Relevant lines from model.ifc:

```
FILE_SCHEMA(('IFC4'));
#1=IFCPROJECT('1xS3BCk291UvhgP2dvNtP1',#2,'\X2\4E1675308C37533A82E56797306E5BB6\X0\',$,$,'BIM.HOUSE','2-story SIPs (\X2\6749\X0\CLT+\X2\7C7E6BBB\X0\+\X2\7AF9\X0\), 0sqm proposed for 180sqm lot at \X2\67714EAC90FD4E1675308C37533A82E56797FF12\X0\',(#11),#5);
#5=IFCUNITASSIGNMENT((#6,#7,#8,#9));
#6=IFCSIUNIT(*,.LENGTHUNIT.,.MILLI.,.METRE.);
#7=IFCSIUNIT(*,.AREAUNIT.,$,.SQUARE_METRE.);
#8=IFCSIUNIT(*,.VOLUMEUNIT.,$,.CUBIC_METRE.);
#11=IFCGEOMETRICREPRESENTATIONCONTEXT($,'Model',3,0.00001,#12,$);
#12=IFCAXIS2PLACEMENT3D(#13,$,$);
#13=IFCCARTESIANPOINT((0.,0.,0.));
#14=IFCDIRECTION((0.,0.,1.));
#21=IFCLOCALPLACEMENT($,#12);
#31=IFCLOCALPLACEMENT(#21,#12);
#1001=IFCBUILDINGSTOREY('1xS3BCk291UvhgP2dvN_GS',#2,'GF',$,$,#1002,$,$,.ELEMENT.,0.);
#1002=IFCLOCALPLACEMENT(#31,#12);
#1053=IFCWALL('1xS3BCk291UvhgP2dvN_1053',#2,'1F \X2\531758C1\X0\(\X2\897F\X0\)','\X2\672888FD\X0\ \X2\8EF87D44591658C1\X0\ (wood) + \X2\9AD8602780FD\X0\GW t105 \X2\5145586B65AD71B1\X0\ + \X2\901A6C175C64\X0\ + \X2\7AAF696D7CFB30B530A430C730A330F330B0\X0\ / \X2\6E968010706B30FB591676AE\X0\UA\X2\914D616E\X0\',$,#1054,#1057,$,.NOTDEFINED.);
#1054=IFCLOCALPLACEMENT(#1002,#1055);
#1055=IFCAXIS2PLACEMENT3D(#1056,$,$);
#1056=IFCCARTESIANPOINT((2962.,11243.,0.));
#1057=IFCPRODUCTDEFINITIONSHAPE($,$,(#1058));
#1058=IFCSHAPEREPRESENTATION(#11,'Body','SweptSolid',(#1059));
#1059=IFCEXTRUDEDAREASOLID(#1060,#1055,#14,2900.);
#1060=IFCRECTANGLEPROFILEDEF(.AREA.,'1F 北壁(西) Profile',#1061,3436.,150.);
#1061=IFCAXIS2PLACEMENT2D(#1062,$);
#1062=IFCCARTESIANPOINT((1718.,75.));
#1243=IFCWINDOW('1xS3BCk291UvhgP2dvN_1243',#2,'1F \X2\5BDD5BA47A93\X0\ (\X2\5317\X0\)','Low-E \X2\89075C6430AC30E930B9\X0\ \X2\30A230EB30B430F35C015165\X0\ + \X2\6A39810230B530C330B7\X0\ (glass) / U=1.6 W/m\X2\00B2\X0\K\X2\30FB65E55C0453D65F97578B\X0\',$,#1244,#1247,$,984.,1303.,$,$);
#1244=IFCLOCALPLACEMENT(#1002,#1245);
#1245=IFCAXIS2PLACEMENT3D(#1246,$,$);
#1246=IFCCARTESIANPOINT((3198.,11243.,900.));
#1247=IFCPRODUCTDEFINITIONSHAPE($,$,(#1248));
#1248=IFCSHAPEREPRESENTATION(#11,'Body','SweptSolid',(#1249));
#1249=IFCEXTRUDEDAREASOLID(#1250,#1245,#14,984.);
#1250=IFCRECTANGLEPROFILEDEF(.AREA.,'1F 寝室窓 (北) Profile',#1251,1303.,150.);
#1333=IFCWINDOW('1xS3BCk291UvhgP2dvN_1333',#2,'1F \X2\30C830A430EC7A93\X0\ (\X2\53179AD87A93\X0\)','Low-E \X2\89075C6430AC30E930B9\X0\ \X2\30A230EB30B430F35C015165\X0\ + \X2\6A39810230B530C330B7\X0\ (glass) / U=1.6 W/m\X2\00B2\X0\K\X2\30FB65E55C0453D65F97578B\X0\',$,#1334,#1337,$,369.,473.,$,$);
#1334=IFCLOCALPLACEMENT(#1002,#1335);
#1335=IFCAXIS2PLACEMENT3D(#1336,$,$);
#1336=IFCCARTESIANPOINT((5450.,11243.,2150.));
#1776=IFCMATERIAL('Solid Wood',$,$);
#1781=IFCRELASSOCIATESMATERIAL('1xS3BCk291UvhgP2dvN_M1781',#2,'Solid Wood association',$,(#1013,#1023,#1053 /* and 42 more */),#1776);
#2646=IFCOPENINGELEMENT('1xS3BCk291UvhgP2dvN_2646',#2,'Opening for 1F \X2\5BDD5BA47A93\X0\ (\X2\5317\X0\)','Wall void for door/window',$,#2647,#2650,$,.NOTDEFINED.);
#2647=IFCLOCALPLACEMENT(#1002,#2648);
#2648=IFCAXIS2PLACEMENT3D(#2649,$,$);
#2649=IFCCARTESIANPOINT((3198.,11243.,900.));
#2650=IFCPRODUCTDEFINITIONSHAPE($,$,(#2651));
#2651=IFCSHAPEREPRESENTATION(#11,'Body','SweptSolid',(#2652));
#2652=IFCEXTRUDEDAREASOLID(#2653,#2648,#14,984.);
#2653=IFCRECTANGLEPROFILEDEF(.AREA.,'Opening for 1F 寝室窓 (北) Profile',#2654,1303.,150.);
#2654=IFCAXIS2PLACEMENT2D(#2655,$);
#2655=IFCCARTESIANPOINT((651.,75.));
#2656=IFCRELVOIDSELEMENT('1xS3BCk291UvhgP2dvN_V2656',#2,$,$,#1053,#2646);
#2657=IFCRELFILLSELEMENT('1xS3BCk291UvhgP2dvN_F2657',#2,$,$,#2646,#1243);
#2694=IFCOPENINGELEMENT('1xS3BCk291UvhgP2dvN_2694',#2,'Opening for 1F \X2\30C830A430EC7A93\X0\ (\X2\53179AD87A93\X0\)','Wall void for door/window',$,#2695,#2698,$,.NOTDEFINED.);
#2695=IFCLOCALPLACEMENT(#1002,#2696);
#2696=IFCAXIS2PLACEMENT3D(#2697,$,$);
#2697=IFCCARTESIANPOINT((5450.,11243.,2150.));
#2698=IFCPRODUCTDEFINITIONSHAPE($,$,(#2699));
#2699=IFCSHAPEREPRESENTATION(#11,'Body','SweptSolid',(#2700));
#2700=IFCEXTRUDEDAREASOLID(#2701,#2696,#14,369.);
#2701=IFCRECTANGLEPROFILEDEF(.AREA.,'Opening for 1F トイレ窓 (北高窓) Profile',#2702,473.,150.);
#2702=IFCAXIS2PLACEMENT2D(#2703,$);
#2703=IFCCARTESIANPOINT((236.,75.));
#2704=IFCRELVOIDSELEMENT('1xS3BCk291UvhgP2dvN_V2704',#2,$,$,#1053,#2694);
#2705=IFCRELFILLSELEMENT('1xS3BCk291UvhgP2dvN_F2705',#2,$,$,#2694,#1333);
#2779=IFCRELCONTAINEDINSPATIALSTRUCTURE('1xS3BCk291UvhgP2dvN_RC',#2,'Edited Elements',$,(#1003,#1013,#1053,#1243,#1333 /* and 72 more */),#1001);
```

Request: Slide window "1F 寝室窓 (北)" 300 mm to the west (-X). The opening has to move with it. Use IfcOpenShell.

```python
import ifcopenshell
import ifcopenshell.api.geometry
import ifcopenshell.util.placement
import ifcopenshell.util.unit

model = ifcopenshell.open("model.ifc")
unit_scale = ifcopenshell.util.unit.calculate_unit_scale(model)

window = model.by_guid("1xS3BCk291UvhgP2dvN_1243")
opening = window.FillsVoids[0].RelatingOpeningElement
wall = opening.VoidsElements[0].RelatingBuildingElement

wall_matrix = ifcopenshell.util.placement.get_local_placement(wall.ObjectPlacement)
shift = wall_matrix[:3, 0] * -0.3 / unit_scale
before = ifcopenshell.util.placement.get_local_placement(window.ObjectPlacement)[:3, 3].copy()

# The window is not placed relative to its opening, so move both.
for product in (opening, window):
    matrix = ifcopenshell.util.placement.get_local_placement(product.ObjectPlacement)
    matrix[:3, 3] += shift
    ifcopenshell.api.geometry.edit_object_placement(model, product=product, matrix=matrix, is_si=False)

after = ifcopenshell.util.placement.get_local_placement(window.ObjectPlacement)[:3, 3]
print("window moved by", (after - before).round(3) + 0.0)

model.write("model_rev.ifc")
```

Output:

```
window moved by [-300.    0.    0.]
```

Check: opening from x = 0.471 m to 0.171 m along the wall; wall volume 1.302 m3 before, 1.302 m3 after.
